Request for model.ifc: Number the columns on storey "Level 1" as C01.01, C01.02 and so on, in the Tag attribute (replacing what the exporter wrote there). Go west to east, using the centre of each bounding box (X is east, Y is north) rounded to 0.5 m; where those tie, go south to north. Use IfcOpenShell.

First a look at what the model holds.

```python
import ifcopenshell
import ifcopenshell.util.element
import ifcopenshell.util.placement

model = ifcopenshell.open("model.ifc")
print(model.schema)
storey = next(s for s in model.by_type("IfcBuildingStorey") if s.Name == "Level 1")
columns = [e for e in ifcopenshell.util.element.get_decomposition(storey) if e.is_a("IfcColumn")]
for e in sorted(columns, key=lambda e: e.id()):
    origin = ifcopenshell.util.placement.get_local_placement(e.ObjectPlacement)[:3, 3]
    print(e.id(), e.Tag, e.Name, origin.round(2) + 0.0, sep=" | ")
```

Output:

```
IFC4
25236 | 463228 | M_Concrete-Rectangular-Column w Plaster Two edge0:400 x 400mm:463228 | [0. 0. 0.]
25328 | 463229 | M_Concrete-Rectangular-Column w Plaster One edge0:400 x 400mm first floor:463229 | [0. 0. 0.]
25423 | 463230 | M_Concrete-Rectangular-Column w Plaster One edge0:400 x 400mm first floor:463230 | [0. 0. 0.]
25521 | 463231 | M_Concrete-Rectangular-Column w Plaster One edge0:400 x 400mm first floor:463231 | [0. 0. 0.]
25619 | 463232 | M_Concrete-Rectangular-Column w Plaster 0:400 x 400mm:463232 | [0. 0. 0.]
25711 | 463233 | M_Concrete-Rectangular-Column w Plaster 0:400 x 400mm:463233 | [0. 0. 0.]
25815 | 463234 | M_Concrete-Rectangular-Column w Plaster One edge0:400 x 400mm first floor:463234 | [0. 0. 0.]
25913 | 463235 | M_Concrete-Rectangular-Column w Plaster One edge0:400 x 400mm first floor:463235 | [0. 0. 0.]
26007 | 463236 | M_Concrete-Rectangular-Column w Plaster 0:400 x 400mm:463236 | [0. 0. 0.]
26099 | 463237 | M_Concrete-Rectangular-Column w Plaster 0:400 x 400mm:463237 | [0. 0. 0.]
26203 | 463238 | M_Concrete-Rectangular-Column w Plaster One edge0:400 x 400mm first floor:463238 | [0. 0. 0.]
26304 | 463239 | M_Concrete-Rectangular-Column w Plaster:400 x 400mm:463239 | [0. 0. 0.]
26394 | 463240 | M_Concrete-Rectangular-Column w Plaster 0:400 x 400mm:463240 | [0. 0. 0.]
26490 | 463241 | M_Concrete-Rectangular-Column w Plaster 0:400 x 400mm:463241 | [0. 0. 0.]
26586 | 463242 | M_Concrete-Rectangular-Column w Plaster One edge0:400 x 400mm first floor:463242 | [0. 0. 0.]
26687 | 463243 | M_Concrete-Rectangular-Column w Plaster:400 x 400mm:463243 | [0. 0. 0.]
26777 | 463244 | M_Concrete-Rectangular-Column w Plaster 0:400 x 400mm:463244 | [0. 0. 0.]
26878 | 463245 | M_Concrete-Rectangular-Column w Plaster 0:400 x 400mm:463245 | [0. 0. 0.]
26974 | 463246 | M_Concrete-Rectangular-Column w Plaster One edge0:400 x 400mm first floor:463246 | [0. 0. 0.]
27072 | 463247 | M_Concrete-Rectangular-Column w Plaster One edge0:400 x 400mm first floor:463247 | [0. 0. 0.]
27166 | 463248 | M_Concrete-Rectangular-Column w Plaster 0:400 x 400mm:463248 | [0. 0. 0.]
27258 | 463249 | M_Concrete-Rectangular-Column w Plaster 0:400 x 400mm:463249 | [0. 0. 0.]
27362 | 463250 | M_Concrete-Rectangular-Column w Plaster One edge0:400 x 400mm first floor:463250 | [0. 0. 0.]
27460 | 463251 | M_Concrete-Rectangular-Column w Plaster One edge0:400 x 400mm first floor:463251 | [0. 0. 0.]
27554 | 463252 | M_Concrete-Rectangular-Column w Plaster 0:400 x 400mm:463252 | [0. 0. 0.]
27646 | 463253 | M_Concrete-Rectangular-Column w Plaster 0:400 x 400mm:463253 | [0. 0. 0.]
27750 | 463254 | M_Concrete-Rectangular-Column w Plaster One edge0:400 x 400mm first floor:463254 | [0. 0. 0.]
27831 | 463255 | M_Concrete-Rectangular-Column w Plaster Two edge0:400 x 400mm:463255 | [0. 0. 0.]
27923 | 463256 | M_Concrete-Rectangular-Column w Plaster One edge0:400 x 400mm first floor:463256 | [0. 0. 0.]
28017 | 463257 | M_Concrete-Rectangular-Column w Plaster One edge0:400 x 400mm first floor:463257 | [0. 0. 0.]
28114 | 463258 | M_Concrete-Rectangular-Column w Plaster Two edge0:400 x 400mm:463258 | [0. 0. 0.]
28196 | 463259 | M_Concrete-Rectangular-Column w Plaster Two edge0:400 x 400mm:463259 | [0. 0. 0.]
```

```python
import ifcopenshell
import ifcopenshell.geom
import ifcopenshell.util.element
import ifcopenshell.util.shape

model = ifcopenshell.open("model.ifc")
settings = ifcopenshell.geom.settings()
settings.set("use-world-coords", True)


def centre(element):
    shape = ifcopenshell.geom.create_shape(settings, element)
    return ifcopenshell.util.shape.get_bbox_centroid(shape.geometry)


storey = next(s for s in model.by_type("IfcBuildingStorey") if s.Name == "Level 1")
columns = [e for e in ifcopenshell.util.element.get_decomposition(storey) if e.is_a("IfcColumn")]

# Insertion points can sit at a corner or the storey origin, so sort by the geometry (in metres).
centres = {e: centre(e) for e in columns}
columns.sort(key=lambda e: (round(centres[e][0] / 0.5), centres[e][1]))

for i, e in enumerate(columns, start=1):
    number = f"C01.{i:02d}"
    e.Tag = number
    print(e.id(), number)

model.write("model_edited.ifc")
```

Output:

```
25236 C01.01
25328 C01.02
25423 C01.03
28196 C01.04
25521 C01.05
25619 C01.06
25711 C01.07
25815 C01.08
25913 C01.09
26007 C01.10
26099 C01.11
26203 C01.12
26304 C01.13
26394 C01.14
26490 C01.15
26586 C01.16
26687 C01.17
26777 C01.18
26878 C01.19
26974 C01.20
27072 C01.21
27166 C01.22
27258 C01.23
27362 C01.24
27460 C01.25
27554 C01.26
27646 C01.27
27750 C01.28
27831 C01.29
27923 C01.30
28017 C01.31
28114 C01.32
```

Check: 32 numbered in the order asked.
